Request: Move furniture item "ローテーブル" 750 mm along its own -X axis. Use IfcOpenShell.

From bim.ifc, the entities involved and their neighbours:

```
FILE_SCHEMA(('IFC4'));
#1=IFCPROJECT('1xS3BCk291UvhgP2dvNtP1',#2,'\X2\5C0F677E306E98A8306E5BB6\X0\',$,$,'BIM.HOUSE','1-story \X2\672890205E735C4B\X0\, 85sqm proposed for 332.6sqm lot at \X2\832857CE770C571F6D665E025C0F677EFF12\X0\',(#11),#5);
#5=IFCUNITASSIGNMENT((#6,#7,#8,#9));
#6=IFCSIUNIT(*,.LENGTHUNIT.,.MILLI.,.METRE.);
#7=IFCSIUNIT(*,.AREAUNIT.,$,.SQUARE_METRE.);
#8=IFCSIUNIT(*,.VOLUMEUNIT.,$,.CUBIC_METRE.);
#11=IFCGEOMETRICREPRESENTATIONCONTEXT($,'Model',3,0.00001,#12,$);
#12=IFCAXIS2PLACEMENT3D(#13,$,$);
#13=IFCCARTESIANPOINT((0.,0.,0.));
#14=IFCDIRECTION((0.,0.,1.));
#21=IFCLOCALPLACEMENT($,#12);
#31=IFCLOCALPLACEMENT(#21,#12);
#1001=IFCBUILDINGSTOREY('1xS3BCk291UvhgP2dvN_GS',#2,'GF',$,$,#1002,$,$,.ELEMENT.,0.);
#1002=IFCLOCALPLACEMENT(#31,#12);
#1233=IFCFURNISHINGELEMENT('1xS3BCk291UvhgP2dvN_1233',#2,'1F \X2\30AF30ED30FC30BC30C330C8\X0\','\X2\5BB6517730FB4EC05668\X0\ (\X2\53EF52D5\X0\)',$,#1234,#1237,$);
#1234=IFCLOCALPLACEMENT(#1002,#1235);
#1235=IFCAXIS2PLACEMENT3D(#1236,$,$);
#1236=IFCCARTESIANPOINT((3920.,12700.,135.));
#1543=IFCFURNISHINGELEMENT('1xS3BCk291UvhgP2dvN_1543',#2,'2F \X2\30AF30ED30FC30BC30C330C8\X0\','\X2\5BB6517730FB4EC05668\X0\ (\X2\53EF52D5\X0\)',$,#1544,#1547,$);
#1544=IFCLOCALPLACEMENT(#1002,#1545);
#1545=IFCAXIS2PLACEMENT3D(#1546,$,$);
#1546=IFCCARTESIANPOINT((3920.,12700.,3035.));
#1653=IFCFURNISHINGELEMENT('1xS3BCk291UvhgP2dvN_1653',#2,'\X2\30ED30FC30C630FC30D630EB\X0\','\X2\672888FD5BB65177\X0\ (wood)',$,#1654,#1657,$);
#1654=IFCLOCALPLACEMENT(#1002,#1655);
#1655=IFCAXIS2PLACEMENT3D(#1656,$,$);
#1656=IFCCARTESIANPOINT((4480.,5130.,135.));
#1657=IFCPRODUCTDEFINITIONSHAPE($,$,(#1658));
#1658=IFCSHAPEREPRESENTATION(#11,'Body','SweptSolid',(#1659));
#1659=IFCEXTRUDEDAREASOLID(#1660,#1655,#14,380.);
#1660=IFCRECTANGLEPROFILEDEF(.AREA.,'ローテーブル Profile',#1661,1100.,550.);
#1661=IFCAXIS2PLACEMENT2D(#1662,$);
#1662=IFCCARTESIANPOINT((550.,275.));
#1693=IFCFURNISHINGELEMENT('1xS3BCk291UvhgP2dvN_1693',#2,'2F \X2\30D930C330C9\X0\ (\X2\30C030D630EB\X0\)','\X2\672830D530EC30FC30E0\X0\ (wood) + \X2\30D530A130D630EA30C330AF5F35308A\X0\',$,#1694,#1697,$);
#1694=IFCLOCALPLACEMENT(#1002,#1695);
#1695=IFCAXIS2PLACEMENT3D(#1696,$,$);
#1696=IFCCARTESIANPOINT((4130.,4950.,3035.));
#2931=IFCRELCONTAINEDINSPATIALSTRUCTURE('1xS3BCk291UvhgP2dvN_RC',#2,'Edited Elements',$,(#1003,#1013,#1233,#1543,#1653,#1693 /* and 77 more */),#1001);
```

```python
import ifcopenshell
import ifcopenshell.api.geometry
import ifcopenshell.util.placement
import ifcopenshell.util.unit

model = ifcopenshell.open("bim.ifc")
unit_scale = ifcopenshell.util.unit.calculate_unit_scale(model)

item = model.by_guid("1xS3BCk291UvhgP2dvN_1653")
matrix = ifcopenshell.util.placement.get_local_placement(item.ObjectPlacement)
matrix[:3, 3] -= matrix[:3, 0] * 0.75 / unit_scale
ifcopenshell.api.geometry.edit_object_placement(model, product=item, matrix=matrix, is_si=False)

print(ifcopenshell.util.placement.get_local_placement(item.ObjectPlacement).round(3) + 0.0)

model.write("bim_v2.ifc")
```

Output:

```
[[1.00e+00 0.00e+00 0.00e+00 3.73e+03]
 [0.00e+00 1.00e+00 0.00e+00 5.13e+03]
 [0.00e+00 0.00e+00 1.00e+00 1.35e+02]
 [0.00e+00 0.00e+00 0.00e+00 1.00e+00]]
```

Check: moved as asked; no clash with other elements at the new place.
